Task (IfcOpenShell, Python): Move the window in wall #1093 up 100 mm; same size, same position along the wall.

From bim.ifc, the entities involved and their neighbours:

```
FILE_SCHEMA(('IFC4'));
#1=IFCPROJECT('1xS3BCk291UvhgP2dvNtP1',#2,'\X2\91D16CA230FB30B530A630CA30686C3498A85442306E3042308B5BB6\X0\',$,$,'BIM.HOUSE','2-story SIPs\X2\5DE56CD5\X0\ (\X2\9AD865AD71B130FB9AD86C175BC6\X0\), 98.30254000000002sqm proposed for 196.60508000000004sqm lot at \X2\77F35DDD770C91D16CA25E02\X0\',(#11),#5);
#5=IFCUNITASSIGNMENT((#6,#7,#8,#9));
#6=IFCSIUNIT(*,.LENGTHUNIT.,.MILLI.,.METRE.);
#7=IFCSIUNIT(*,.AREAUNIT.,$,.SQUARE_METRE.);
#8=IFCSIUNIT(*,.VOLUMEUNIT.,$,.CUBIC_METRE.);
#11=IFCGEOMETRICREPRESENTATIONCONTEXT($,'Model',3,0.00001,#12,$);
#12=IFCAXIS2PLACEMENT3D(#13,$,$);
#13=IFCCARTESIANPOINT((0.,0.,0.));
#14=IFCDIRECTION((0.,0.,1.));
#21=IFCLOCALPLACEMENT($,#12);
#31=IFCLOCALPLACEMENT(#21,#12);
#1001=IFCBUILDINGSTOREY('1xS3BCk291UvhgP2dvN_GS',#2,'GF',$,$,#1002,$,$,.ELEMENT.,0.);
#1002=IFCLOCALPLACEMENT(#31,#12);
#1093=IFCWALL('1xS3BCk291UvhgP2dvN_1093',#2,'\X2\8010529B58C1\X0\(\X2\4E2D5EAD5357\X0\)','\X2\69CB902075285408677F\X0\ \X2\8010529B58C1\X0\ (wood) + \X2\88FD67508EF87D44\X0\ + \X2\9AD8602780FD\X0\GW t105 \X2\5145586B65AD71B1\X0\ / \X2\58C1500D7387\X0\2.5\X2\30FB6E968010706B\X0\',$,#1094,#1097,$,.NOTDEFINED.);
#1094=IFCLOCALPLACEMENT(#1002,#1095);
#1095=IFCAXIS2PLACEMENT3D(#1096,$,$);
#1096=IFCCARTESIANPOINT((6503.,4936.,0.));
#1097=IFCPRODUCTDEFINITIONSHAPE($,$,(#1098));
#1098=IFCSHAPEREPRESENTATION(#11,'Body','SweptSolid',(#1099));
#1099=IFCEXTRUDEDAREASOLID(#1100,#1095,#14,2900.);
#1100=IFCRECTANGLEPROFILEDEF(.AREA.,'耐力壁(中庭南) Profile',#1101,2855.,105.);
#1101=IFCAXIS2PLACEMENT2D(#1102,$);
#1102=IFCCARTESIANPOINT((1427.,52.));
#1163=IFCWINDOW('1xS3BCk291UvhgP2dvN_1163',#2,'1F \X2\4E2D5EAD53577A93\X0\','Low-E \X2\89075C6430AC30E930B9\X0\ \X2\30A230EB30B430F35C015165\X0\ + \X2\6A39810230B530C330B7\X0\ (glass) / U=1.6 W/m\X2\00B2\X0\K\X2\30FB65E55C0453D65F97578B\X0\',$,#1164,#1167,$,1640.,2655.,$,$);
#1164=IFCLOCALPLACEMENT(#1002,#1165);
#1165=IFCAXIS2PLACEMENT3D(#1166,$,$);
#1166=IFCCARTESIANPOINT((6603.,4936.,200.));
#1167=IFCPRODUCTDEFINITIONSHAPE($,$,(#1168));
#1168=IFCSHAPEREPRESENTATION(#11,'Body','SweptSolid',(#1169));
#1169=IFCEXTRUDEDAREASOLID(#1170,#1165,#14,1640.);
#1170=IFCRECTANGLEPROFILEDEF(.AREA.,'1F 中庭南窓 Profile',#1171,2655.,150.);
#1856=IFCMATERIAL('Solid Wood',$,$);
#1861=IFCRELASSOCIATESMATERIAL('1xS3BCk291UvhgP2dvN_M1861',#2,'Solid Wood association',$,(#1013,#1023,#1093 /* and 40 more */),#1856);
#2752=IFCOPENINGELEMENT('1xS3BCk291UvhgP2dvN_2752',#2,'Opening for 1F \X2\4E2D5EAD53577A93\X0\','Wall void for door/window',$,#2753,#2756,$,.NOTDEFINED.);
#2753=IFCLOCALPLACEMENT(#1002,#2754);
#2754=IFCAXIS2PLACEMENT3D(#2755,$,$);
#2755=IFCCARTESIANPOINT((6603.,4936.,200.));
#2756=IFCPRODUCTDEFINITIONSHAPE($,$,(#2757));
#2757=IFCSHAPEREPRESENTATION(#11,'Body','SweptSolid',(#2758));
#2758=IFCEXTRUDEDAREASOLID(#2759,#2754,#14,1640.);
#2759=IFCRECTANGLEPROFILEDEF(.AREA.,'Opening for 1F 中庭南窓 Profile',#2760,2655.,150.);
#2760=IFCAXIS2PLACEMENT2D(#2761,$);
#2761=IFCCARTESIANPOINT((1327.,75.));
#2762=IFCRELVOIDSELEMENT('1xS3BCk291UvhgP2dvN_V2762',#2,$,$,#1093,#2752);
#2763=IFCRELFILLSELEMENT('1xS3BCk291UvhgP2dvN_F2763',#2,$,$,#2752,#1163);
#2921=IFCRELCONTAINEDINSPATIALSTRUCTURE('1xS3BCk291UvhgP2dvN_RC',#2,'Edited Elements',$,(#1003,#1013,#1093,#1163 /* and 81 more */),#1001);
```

```python
import numpy as np
import ifcopenshell
import ifcopenshell.api.geometry
import ifcopenshell.util.placement
import ifcopenshell.util.unit

model = ifcopenshell.open("bim.ifc")
unit_scale = ifcopenshell.util.unit.calculate_unit_scale(model)

window = model.by_guid("1xS3BCk291UvhgP2dvN_1163")
opening = window.FillsVoids[0].RelatingOpeningElement
dz = 100.0

shift = np.array([0.0, 0.0, dz])
# The window is not placed relative to its opening, so move both.
for product in (opening, window):
    matrix = ifcopenshell.util.placement.get_local_placement(product.ObjectPlacement)
    matrix[:3, 3] += shift
    ifcopenshell.api.geometry.edit_object_placement(model, product=product, matrix=matrix, is_si=False)

print(f"moved by {dz * unit_scale:+.3f} m")

model.write("bim-out.ifc")
```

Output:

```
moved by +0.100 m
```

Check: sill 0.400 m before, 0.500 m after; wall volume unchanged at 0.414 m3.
